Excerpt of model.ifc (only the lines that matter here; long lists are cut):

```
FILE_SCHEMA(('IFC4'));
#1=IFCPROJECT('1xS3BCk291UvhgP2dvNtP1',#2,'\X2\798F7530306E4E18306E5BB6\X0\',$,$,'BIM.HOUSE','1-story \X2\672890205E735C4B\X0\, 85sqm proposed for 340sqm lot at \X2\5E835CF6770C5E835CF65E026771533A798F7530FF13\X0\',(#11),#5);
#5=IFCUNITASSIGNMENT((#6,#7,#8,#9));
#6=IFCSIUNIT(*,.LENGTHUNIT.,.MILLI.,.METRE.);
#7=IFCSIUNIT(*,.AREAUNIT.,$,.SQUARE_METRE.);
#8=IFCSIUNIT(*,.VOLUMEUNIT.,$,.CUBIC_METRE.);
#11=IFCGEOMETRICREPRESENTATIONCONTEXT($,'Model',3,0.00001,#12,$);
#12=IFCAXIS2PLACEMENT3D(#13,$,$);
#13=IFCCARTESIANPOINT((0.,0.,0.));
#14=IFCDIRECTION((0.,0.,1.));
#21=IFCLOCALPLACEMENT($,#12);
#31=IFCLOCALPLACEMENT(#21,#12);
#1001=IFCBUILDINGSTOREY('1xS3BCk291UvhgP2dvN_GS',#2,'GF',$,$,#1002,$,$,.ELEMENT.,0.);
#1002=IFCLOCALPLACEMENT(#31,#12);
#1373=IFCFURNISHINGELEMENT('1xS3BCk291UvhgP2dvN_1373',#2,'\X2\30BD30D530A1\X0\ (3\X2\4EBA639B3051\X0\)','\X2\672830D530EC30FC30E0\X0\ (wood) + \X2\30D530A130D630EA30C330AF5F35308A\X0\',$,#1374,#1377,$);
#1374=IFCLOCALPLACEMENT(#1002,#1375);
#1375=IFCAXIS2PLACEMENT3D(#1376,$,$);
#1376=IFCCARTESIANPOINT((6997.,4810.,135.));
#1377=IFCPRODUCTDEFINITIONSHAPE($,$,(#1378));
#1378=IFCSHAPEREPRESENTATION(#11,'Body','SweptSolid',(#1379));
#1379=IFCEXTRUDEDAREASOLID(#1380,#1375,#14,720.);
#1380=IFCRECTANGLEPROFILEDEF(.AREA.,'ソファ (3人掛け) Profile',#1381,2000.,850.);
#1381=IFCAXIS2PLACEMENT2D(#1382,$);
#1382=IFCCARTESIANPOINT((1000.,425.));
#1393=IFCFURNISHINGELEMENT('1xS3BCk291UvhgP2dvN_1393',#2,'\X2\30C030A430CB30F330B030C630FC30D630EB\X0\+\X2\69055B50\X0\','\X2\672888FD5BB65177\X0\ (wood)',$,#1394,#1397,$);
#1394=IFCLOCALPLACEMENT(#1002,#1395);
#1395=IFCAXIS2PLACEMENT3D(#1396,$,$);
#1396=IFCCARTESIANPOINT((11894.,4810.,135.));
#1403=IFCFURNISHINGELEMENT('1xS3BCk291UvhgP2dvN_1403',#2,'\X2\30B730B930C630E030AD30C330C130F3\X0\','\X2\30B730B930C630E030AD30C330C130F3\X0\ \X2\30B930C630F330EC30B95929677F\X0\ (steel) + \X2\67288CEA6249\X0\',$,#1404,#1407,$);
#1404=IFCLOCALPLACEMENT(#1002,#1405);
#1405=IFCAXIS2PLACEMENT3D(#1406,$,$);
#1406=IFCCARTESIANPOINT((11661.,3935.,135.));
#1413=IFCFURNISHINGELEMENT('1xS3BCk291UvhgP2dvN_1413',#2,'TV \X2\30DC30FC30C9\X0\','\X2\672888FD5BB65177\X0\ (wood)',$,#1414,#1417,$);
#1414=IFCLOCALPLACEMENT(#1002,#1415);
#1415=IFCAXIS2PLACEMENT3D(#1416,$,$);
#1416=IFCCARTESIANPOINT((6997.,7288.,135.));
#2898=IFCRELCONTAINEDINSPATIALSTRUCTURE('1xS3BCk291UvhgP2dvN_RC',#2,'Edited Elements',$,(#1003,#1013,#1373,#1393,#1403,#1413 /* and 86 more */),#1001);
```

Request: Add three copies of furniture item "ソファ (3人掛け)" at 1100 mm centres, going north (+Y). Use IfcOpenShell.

```python
import numpy as np
import ifcopenshell
import ifcopenshell.api.geometry
import ifcopenshell.api.root
import ifcopenshell.util.element
import ifcopenshell.util.placement

model = ifcopenshell.open("model.ifc")


def reuse_history(source, copy):
    """copy_class also copies each property set's owner history, people and application; keep the originals."""
    for rel in copy.IsDefinedBy:
        if rel.is_a("IfcRelDefinesByProperties") and (history := rel.RelatingPropertyDefinition.OwnerHistory):
            rel.RelatingPropertyDefinition.OwnerHistory = source.OwnerHistory
            ifcopenshell.util.element.remove_deep2(model, history)


source = model.by_guid("1xS3BCk291UvhgP2dvN_1373")
base = ifcopenshell.util.placement.get_local_placement(source.ObjectPlacement)
step = np.array([0.0, 1.0, 0.0]) * 1100.0

for i in range(1, 4):
    copy = ifcopenshell.api.root.copy_class(model, product=source)
    copy.Representation = ifcopenshell.util.element.copy_deep(
        model, source.Representation, exclude=["IfcGeometricRepresentationContext", "IfcRepresentationMap"]
    )
    reuse_history(source, copy)
    matrix = base.copy()
    matrix[:3, 3] += i * step
    print("added at", matrix[:3, 3].round(3) + 0.0)
    ifcopenshell.api.geometry.edit_object_placement(model, product=copy, matrix=matrix, is_si=False)

model.write("model-out.ifc")
```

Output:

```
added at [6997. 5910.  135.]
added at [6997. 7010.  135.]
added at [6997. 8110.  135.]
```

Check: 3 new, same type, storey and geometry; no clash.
